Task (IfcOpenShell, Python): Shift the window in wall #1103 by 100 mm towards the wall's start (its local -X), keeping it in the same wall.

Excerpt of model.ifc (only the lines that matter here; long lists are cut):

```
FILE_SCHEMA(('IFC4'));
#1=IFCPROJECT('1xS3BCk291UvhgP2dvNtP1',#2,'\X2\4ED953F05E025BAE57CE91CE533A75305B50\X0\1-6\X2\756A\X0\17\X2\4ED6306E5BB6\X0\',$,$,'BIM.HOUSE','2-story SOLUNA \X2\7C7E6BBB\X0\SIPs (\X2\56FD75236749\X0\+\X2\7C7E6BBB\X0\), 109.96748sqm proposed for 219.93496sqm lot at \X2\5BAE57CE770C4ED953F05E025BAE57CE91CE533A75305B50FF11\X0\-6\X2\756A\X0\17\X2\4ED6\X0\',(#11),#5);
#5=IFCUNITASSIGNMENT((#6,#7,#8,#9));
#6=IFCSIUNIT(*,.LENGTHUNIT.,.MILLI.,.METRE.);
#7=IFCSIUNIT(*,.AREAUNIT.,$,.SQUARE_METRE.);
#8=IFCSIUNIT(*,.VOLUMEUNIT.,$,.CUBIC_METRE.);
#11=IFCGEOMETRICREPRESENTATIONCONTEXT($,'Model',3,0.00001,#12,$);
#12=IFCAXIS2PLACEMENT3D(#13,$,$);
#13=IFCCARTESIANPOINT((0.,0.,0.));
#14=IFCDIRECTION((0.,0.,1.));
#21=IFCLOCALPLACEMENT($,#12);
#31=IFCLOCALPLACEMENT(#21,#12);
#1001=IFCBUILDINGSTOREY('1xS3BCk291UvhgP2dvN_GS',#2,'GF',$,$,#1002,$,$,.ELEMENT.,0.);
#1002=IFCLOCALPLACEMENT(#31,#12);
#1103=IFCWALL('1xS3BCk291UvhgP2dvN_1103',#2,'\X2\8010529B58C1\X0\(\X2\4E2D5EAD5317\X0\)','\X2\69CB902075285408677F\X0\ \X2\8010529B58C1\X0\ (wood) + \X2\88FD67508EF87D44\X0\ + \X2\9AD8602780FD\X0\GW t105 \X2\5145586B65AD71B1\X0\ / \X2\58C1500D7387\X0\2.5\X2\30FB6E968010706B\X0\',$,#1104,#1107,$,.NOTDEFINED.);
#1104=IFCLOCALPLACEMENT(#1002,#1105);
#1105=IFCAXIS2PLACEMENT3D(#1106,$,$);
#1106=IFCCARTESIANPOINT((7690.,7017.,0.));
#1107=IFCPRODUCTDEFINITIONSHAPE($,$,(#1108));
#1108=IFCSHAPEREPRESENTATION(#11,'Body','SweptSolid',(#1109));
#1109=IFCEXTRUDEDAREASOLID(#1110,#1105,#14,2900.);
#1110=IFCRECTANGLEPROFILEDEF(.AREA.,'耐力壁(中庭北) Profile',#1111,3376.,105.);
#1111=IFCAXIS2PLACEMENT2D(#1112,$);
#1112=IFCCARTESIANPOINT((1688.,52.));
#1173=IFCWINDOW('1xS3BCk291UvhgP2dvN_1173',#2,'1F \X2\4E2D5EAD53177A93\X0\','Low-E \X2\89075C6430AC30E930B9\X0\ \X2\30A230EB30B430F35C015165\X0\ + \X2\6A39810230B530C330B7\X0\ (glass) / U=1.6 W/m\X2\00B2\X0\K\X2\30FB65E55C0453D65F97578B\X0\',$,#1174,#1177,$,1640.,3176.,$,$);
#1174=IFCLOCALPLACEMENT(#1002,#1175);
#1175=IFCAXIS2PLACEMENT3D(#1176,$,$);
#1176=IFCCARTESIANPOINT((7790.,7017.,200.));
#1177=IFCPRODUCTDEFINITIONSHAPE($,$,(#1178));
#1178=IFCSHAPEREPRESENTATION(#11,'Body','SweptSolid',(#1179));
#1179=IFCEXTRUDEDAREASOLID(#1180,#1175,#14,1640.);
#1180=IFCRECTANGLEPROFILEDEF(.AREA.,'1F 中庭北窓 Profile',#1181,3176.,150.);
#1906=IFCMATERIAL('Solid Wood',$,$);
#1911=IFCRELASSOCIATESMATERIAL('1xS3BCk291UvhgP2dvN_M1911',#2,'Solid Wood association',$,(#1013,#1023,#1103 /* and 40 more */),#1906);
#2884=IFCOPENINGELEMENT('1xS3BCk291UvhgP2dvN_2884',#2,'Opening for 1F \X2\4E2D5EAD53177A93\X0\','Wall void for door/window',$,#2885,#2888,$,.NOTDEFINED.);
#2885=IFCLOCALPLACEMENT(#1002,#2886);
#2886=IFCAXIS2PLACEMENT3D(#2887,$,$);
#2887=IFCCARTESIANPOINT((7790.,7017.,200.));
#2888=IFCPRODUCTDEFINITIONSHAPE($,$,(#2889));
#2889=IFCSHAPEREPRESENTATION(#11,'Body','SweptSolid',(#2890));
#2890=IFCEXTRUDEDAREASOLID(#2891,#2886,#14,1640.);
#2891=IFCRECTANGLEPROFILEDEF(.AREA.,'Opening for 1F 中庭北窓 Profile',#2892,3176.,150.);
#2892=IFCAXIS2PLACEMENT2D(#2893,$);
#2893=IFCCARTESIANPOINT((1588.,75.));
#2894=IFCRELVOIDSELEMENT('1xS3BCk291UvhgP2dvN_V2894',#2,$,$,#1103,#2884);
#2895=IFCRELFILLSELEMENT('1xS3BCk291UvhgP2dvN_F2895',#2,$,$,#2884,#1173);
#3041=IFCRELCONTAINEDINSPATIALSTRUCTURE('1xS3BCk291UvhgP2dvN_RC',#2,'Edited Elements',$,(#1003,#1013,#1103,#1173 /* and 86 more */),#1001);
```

```python
import ifcopenshell
import ifcopenshell.api.geometry
import ifcopenshell.util.placement

model = ifcopenshell.open("model.ifc")

window = model.by_guid("1xS3BCk291UvhgP2dvN_1173")
opening = window.FillsVoids[0].RelatingOpeningElement
wall = opening.VoidsElements[0].RelatingBuildingElement

wall_matrix = ifcopenshell.util.placement.get_local_placement(wall.ObjectPlacement)
shift = wall_matrix[:3, 0] * -100.0
before = ifcopenshell.util.placement.get_local_placement(window.ObjectPlacement)[:3, 3].copy()

# The window is not placed relative to its opening, so move both.
for product in (opening, window):
    matrix = ifcopenshell.util.placement.get_local_placement(product.ObjectPlacement)
    matrix[:3, 3] += shift
    ifcopenshell.api.geometry.edit_object_placement(model, product=product, matrix=matrix, is_si=False)

after = ifcopenshell.util.placement.get_local_placement(window.ObjectPlacement)[:3, 3]
print("window moved by", (after - before).round(3) + 0.0)

model.write("model_rev.ifc")
```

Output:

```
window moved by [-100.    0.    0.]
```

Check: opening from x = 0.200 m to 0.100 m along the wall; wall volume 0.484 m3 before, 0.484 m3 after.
